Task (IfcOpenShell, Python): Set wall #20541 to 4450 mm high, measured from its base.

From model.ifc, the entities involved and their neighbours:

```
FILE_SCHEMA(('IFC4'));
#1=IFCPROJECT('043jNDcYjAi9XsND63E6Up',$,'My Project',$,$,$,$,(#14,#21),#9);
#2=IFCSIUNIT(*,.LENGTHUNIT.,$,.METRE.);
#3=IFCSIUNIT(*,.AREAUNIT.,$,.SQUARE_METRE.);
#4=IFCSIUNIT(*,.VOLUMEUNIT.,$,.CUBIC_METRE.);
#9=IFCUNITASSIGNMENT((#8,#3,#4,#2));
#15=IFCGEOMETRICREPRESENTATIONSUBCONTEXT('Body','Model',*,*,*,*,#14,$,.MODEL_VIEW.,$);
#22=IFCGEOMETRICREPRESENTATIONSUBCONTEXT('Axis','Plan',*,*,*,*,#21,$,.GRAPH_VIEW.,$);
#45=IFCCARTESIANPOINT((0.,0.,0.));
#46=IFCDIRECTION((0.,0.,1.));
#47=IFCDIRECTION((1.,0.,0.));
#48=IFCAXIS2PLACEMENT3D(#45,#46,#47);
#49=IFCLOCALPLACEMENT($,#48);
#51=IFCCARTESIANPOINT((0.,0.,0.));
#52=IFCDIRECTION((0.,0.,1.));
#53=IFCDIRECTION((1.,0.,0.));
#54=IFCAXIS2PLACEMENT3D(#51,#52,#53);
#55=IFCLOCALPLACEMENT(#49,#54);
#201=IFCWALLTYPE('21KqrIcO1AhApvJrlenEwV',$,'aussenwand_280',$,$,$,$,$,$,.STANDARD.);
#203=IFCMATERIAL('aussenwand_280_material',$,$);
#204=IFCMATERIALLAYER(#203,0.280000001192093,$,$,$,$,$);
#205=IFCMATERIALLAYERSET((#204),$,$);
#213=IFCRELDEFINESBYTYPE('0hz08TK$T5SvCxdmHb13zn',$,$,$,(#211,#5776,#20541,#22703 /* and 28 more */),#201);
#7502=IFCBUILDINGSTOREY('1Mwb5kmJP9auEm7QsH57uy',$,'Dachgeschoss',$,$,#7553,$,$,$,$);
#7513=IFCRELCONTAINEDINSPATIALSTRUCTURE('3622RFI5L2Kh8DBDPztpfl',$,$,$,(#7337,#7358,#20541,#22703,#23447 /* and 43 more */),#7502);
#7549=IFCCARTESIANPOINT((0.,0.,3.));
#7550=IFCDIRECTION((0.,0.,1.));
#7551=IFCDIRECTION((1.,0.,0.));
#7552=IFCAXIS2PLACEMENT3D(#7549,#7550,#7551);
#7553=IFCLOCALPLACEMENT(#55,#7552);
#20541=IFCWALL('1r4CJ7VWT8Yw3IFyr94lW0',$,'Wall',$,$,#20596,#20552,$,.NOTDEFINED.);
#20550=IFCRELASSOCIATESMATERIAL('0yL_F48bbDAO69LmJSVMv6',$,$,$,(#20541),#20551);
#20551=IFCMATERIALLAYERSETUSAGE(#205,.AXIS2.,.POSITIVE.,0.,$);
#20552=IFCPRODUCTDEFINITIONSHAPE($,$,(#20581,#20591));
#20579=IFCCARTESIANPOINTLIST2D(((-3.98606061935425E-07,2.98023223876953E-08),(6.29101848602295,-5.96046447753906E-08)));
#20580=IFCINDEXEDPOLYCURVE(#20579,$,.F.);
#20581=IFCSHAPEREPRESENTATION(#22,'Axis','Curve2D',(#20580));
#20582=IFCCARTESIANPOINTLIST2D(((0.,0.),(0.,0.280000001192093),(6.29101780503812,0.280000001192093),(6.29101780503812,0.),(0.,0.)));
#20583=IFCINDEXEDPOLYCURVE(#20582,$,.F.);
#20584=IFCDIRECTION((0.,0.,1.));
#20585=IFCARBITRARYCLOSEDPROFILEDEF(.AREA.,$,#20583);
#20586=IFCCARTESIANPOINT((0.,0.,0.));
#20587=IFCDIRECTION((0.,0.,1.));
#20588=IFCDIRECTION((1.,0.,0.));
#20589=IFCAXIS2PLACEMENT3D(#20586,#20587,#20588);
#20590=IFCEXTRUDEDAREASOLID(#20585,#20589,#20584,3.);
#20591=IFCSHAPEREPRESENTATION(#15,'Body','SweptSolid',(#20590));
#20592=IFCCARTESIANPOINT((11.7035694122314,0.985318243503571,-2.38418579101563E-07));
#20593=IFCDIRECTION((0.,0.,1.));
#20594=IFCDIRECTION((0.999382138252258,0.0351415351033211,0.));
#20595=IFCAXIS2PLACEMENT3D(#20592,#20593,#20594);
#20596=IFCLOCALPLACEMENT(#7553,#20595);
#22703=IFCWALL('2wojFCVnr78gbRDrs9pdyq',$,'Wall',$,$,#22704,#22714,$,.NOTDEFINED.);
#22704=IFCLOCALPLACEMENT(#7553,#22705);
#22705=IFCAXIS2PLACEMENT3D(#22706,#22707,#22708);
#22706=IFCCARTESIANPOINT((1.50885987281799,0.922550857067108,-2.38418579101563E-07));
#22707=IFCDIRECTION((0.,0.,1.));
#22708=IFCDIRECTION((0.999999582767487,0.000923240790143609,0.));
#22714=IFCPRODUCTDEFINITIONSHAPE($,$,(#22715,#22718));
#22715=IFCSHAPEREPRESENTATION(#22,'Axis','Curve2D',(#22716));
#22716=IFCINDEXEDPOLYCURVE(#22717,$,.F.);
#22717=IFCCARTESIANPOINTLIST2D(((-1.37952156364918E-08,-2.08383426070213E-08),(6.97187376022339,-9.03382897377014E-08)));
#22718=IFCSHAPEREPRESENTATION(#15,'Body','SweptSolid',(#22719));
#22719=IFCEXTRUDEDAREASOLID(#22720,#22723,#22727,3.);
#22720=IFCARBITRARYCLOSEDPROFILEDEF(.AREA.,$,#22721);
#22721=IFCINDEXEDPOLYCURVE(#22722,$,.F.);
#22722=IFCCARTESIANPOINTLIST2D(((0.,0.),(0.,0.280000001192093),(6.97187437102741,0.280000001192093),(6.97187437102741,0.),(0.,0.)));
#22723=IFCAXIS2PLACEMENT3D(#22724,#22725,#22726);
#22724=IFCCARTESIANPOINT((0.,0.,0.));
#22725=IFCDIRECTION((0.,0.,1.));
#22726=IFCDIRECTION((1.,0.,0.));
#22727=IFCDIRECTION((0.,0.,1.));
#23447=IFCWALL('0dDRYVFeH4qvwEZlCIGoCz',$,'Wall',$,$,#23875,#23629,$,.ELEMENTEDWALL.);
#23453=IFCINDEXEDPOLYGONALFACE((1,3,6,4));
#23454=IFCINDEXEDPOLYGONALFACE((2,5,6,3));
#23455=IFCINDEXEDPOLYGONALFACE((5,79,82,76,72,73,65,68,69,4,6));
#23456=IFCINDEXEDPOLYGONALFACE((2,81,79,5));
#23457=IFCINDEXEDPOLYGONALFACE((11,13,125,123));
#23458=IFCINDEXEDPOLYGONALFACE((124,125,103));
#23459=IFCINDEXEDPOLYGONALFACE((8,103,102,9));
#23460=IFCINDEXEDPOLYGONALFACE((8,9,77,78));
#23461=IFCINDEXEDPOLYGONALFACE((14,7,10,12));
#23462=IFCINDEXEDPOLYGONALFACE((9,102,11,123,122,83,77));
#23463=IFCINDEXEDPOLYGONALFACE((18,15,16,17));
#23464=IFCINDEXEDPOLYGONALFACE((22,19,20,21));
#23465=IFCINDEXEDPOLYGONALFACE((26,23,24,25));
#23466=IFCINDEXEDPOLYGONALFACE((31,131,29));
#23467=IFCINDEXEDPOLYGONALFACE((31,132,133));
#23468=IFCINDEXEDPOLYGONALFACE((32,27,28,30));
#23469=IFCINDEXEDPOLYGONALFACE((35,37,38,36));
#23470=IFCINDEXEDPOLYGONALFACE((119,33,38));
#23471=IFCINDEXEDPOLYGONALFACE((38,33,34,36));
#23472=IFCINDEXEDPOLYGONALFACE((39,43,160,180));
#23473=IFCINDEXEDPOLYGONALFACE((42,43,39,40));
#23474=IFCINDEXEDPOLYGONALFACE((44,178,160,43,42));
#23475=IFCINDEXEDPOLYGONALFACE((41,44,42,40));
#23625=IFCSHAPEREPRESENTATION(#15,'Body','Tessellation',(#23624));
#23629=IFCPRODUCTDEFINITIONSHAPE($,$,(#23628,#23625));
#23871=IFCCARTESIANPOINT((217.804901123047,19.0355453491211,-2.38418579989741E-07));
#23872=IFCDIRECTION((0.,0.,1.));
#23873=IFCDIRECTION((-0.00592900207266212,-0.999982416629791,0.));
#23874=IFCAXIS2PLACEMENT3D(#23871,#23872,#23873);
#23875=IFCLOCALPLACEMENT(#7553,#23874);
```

```python
import ifcopenshell
import ifcopenshell.geom
import ifcopenshell.util.representation
import ifcopenshell.util.shape
import ifcopenshell.util.unit

model = ifcopenshell.open("model.ifc")
unit_scale = ifcopenshell.util.unit.calculate_unit_scale(model)
settings = ifcopenshell.geom.settings()


def volume(element):
    """Net volume in cubic metres, openings subtracted."""
    shape = ifcopenshell.geom.create_shape(settings, element)
    return ifcopenshell.util.shape.get_volume(shape.geometry)


wall = model.by_id(20541)
before = volume(wall)

body = ifcopenshell.util.representation.get_representation(wall, "Model", "Body")
solid = body.Items[0]
old_height = solid.Depth
solid.Depth = 4.45 / unit_scale
after = volume(wall)

print(f"height {old_height:g} -> {solid.Depth:g}, volume {before:.3f} -> {after:.3f} m3")

model.write("model_v2.ifc")
```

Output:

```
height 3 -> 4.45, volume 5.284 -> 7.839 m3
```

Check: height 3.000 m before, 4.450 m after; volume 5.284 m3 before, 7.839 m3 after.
